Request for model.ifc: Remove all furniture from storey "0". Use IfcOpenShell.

First a look at what the model holds.

```python
import ifcopenshell
import ifcopenshell.util.element

model = ifcopenshell.open("model.ifc")
print(model.schema)
storey = next(s for s in model.by_type("IfcBuildingStorey") if s.Name == "0")
furniture = [e for e in ifcopenshell.util.element.get_decomposition(storey) if e.is_a("IfcFurnishingElement")]
seen = {}
for e in furniture:
    element_type = ifcopenshell.util.element.get_type(e)
    name = element_type.Name if element_type not in (None, e) else None
    seen[name] = seen.get(name, 0) + 1
for name, count in sorted(seen.items(), key=str):
    print(count, "x", name)
```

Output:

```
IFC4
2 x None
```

```python
import ifcopenshell
import ifcopenshell.api.root
import ifcopenshell.util.element

model = ifcopenshell.open("model.ifc")

storey = next(s for s in model.by_type("IfcBuildingStorey") if s.Name == "0")
furniture = [e for e in ifcopenshell.util.element.get_decomposition(storey) if e.is_a("IfcFurnishingElement")]

for e in furniture:
    ifcopenshell.api.root.remove_product(model, product=e)
print(len(furniture), "removed")

model.write("model_edited.ifc")
```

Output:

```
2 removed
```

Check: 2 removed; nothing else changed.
